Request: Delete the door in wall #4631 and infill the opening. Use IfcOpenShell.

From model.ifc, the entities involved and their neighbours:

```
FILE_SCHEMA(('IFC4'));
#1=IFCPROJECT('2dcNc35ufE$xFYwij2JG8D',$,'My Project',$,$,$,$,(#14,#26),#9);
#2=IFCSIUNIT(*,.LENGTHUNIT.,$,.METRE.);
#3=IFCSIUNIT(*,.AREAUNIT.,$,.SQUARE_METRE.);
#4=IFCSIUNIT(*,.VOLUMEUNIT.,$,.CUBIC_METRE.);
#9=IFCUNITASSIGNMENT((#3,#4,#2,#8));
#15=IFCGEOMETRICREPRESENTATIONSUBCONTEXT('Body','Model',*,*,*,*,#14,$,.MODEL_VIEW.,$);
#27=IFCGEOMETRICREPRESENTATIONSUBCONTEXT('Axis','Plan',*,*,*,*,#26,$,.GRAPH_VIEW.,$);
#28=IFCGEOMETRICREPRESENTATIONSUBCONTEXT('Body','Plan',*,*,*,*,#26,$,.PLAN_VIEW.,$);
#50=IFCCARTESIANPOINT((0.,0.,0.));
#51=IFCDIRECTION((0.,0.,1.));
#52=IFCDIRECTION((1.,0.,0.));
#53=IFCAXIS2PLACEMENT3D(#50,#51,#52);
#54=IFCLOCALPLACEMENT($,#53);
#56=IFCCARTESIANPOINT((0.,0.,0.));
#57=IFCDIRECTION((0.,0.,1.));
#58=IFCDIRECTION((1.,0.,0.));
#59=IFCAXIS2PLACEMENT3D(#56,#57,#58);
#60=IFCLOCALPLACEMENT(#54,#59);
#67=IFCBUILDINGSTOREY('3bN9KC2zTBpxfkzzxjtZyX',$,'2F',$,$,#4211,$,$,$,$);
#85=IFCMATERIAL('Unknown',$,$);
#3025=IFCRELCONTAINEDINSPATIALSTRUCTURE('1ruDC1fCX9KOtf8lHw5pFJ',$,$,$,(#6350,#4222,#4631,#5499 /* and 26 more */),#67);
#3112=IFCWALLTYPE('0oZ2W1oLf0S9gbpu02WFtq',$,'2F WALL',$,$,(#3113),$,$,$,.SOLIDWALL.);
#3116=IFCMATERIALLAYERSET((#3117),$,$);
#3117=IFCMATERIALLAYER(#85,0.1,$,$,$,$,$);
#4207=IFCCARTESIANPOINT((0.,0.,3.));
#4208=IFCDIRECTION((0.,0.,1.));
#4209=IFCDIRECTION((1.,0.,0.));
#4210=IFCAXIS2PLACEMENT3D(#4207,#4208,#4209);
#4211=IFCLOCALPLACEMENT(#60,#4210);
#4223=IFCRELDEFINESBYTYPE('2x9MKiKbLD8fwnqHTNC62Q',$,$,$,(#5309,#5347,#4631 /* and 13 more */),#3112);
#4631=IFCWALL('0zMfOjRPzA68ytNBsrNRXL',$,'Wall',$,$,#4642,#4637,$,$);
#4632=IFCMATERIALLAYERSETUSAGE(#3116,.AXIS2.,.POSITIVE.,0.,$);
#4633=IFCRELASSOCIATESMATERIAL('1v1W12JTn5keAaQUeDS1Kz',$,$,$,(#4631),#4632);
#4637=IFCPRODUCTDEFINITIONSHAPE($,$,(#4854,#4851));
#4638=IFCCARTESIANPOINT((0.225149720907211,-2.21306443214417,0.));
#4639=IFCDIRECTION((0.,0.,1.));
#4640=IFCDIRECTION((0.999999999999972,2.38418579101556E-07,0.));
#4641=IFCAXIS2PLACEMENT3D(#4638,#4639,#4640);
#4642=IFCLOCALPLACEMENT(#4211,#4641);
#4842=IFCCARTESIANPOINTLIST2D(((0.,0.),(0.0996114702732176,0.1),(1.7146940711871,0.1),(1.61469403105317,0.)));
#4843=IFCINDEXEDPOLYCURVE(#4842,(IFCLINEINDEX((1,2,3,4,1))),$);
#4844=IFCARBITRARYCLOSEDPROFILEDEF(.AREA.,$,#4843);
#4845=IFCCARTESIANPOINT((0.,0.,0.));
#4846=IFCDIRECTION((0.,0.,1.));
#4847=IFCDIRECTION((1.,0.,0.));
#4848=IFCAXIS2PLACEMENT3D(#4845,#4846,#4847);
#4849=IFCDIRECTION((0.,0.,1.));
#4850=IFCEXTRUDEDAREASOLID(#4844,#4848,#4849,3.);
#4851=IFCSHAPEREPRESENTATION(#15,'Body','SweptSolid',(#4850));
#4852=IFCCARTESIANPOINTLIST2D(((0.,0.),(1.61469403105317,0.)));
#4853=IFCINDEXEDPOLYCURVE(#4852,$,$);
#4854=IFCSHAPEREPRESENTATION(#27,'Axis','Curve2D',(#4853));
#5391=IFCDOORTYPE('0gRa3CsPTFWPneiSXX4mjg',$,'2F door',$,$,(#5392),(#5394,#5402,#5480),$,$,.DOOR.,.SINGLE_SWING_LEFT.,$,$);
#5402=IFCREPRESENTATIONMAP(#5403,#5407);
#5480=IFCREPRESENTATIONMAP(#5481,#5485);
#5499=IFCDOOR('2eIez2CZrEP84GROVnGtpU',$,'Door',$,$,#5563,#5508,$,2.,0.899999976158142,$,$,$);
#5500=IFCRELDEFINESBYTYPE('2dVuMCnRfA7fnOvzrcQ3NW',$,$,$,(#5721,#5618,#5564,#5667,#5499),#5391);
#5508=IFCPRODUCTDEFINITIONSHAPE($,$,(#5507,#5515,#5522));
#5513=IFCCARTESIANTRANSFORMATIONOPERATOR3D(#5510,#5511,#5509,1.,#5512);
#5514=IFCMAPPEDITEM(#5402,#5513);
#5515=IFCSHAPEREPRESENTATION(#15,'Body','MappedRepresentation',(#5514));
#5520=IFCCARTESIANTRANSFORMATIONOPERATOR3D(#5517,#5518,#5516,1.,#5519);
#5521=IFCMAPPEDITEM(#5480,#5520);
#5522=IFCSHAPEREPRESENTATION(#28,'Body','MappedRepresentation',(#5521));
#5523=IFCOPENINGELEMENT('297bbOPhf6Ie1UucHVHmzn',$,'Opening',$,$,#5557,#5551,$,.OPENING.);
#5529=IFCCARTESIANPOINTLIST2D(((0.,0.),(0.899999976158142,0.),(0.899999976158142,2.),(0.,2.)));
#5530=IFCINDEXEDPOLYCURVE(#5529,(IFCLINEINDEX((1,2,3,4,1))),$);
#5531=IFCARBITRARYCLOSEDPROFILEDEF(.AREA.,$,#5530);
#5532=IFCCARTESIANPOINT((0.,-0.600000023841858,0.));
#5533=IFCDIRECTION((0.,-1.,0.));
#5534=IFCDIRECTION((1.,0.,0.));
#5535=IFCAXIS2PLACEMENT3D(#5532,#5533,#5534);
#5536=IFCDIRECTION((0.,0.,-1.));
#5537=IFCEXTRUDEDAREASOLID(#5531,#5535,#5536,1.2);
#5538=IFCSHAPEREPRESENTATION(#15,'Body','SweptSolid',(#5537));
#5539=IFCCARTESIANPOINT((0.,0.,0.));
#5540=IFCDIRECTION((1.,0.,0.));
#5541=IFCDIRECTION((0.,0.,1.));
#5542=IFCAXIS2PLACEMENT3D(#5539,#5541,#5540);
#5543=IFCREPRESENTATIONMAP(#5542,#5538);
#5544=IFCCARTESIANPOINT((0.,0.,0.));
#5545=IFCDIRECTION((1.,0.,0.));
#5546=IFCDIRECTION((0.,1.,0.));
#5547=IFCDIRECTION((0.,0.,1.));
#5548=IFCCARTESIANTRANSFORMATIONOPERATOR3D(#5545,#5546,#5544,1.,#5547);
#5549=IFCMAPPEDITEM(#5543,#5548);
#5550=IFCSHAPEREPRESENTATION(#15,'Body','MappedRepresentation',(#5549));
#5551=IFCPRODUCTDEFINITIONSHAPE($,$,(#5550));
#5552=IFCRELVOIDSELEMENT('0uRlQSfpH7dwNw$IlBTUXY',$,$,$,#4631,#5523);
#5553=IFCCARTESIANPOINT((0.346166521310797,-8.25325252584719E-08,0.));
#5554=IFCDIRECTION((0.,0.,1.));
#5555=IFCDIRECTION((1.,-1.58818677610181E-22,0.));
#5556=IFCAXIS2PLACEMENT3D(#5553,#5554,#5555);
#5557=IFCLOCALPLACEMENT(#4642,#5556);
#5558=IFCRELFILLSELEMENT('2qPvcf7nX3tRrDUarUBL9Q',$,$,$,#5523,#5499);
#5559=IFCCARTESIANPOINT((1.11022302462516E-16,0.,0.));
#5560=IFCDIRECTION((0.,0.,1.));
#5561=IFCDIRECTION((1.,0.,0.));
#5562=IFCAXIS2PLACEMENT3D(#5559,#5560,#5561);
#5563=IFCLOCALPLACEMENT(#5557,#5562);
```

```python
import ifcopenshell
import ifcopenshell.api.feature
import ifcopenshell.api.root
import ifcopenshell.geom
import ifcopenshell.util.shape

model = ifcopenshell.open("model.ifc")
settings = ifcopenshell.geom.settings()


def volume(element):
    """Net volume in cubic metres, openings subtracted."""
    shape = ifcopenshell.geom.create_shape(settings, element)
    return ifcopenshell.util.shape.get_volume(shape.geometry)


door = model.by_id(5499)
opening = door.FillsVoids[0].RelatingOpeningElement
wall = opening.VoidsElements[0].RelatingBuildingElement
before = volume(wall)

ifcopenshell.api.root.remove_product(model, product=door)
ifcopenshell.api.feature.remove_feature(model, feature=opening)

after = volume(wall)

print(f"wall volume {before:.3f} -> {after:.3f} m3")

model.write("model-out.ifc")
```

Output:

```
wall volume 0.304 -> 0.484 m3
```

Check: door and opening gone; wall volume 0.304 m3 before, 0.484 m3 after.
